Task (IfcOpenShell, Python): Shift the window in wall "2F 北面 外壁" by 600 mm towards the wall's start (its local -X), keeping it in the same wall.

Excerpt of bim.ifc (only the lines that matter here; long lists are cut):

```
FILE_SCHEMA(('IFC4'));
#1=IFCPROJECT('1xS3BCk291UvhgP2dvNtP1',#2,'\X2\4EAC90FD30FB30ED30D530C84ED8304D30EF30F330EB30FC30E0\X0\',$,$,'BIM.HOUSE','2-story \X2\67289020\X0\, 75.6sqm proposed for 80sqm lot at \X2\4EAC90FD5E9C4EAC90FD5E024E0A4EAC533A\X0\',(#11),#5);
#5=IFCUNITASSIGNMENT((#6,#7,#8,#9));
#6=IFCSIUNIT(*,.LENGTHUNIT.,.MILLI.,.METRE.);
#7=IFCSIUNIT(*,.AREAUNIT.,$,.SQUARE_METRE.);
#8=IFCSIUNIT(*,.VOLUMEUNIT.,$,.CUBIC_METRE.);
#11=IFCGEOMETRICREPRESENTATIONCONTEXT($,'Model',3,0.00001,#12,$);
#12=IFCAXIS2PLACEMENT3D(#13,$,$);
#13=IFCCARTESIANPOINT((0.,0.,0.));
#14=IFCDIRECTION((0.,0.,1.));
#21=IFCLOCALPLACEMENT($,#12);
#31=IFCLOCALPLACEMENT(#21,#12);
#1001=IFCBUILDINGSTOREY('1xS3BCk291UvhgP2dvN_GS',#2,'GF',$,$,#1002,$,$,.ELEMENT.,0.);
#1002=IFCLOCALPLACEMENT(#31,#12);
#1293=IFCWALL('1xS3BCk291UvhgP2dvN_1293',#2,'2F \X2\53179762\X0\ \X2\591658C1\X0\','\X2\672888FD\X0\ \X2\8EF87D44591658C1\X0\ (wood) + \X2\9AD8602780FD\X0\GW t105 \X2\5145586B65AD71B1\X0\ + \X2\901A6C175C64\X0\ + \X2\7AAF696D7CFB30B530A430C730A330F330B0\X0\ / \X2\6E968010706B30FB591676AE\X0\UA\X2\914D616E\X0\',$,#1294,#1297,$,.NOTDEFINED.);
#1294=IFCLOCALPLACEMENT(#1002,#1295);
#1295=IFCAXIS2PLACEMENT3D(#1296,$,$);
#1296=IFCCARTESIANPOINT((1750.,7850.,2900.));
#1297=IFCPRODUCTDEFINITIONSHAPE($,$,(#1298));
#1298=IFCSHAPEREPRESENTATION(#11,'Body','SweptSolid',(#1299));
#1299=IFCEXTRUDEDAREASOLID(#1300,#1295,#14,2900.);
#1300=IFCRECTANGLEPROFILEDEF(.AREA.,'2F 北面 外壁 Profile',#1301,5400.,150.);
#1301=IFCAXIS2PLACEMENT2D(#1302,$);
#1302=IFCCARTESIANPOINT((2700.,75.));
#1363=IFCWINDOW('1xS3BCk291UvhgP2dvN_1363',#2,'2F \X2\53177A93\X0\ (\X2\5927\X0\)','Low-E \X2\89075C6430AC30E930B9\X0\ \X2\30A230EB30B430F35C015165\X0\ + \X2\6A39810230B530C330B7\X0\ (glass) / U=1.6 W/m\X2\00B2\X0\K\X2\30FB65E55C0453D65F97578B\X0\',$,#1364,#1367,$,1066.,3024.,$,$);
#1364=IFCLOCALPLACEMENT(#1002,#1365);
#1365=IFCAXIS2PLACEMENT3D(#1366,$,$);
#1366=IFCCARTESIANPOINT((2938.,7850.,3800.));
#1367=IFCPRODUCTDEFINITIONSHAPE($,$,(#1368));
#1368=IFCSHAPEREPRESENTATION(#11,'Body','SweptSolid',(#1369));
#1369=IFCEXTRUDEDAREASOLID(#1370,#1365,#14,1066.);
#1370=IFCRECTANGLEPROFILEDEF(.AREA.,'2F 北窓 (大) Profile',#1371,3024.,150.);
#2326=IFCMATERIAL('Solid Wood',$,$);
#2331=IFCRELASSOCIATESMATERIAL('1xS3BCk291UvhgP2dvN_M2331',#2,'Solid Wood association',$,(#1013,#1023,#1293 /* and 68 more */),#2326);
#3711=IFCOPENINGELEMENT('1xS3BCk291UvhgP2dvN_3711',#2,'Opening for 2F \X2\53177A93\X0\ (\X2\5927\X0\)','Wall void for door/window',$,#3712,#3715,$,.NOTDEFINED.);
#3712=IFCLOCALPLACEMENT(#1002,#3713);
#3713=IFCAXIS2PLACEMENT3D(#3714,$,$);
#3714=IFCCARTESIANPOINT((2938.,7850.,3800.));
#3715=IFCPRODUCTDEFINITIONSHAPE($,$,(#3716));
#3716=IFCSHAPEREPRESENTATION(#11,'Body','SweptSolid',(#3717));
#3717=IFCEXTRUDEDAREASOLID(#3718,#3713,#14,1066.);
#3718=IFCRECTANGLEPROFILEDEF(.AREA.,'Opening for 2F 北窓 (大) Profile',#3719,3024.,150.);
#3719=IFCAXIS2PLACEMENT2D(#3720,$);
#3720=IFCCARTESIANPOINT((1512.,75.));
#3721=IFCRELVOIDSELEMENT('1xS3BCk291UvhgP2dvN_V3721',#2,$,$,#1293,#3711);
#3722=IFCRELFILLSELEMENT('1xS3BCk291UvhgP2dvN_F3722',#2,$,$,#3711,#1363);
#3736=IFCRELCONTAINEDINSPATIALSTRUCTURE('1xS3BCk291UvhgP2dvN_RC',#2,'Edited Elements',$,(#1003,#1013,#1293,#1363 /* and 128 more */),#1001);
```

```python
import ifcopenshell
import ifcopenshell.api.geometry
import ifcopenshell.util.placement
import ifcopenshell.util.unit

model = ifcopenshell.open("bim.ifc")
unit_scale = ifcopenshell.util.unit.calculate_unit_scale(model)

window = model.by_guid("1xS3BCk291UvhgP2dvN_1363")
opening = window.FillsVoids[0].RelatingOpeningElement
wall = opening.VoidsElements[0].RelatingBuildingElement

wall_matrix = ifcopenshell.util.placement.get_local_placement(wall.ObjectPlacement)
shift = wall_matrix[:3, 0] * -0.6 / unit_scale
before = ifcopenshell.util.placement.get_local_placement(window.ObjectPlacement)[:3, 3].copy()

# The window is not placed relative to its opening, so move both.
for product in (opening, window):
    matrix = ifcopenshell.util.placement.get_local_placement(product.ObjectPlacement)
    matrix[:3, 3] += shift
    ifcopenshell.api.geometry.edit_object_placement(model, product=product, matrix=matrix, is_si=False)

after = ifcopenshell.util.placement.get_local_placement(window.ObjectPlacement)[:3, 3]
print("window moved by", (after - before).round(3) + 0.0)

model.write("bim_v2.ifc")
```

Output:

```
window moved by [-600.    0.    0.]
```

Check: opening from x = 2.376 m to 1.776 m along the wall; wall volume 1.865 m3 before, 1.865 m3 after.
